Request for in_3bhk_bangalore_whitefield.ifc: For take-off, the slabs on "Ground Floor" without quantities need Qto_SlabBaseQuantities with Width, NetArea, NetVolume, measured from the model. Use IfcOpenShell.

First a look at what the model holds.

```python
import ifcopenshell
import ifcopenshell.util.element
import ifcopenshell.util.unit

model = ifcopenshell.open("in_3bhk_bangalore_whitefield.ifc")
print(model.schema)
for unit_type in ("LENGTHUNIT", "AREAUNIT", "VOLUMEUNIT"):
    print(unit_type, ifcopenshell.util.unit.calculate_unit_scale(model, unit_type))
storey = next(s for s in model.by_type("IfcBuildingStorey") if s.Name == "Ground Floor")
slabs = [e for e in ifcopenshell.util.element.get_decomposition(storey) if e.is_a("IfcSlab")]
for e in sorted(slabs, key=lambda e: e.id()):
    print(e.id(), e.is_a(), e.Name, list(ifcopenshell.util.element.get_psets(e, qtos_only=True)), sep=" | ")
```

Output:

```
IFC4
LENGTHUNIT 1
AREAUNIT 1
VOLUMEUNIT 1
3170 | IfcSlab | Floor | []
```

```python
import ifcopenshell
import ifcopenshell.api.pset
import ifcopenshell.geom
import ifcopenshell.util.element
import ifcopenshell.util.shape
import ifcopenshell.util.unit

model = ifcopenshell.open("in_3bhk_bangalore_whitefield.ifc")
unit_scale = ifcopenshell.util.unit.calculate_unit_scale(model)
area_scale = ifcopenshell.util.unit.calculate_unit_scale(model, "AREAUNIT")
volume_scale = ifcopenshell.util.unit.calculate_unit_scale(model, "VOLUMEUNIT")
settings = ifcopenshell.geom.settings()

storey = next(s for s in model.by_type("IfcBuildingStorey") if s.Name == "Ground Floor")
slabs = [e for e in ifcopenshell.util.element.get_decomposition(storey) if e.is_a("IfcSlab")]

for e in sorted(slabs, key=lambda e: e.id()):
    if ifcopenshell.util.element.get_psets(e, qtos_only=True, should_inherit=False):
        continue
    # Geometry comes back in metres, in the element's own axes.
    shape = ifcopenshell.geom.create_shape(settings, e)
    values = {
        "Width": ifcopenshell.util.shape.get_z(shape.geometry) / unit_scale,
        "NetArea": ifcopenshell.util.shape.get_footprint_area(shape.geometry) / area_scale,
        "NetVolume": ifcopenshell.util.shape.get_volume(shape.geometry) / volume_scale,
    }
    qto = ifcopenshell.api.pset.add_qto(model, product=e, name="Qto_SlabBaseQuantities")
    ifcopenshell.api.pset.edit_qto(model, qto=qto, properties=values)
    print(e.id(), {k: round(v, 3) for k, v in values.items()})

model.write("in_3bhk_bangalore_whitefield_edited.ifc")
```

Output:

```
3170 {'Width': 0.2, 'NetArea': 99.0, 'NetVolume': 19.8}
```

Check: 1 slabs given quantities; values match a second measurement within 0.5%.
